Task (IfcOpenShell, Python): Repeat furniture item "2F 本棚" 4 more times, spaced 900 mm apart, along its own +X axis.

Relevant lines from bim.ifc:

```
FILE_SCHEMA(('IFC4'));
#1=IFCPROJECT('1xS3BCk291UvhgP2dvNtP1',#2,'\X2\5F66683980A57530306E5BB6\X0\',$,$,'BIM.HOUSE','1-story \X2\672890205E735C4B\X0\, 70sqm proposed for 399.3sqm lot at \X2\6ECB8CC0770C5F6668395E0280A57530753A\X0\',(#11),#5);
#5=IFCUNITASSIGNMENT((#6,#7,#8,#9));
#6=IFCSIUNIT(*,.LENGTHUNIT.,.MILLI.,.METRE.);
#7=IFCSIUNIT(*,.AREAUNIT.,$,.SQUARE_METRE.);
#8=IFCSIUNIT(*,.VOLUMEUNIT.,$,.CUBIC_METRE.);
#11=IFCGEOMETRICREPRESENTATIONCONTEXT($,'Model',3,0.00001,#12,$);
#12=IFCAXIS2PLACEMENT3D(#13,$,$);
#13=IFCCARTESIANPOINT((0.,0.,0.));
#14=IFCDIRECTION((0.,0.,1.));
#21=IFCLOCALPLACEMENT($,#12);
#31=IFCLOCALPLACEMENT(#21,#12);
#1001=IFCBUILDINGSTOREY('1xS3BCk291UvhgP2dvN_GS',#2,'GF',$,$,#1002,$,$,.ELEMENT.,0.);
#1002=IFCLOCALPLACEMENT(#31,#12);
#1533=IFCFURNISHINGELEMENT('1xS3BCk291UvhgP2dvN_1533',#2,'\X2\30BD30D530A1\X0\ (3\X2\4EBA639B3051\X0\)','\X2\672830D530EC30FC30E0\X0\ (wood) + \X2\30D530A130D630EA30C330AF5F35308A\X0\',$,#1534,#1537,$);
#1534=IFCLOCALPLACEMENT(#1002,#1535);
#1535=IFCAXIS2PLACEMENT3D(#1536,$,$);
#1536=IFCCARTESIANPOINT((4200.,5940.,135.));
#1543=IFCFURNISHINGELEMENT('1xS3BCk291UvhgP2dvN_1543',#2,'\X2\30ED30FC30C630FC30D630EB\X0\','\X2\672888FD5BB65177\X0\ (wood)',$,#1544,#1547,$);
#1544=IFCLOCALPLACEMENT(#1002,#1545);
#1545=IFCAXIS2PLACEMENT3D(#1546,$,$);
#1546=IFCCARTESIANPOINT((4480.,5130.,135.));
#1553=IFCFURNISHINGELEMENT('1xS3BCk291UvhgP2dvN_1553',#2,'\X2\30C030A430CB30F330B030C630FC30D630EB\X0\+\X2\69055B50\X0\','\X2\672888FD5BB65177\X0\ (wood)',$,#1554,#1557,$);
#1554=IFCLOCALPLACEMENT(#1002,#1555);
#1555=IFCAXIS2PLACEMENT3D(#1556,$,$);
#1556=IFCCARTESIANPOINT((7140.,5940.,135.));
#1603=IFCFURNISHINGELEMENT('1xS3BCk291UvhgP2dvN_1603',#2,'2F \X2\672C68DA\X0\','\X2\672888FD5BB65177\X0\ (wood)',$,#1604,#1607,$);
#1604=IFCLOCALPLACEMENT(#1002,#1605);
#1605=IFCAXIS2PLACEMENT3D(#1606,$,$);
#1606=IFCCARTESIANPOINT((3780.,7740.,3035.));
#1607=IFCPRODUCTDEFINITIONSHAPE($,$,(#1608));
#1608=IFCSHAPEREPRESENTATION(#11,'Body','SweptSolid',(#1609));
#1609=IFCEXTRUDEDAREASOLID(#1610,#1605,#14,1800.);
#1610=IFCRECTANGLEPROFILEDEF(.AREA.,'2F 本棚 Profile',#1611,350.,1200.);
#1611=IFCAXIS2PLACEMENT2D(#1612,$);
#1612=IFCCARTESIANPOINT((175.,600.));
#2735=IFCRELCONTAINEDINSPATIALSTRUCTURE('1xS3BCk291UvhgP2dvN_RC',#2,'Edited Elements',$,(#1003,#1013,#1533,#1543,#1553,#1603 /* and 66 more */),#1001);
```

```python
import ifcopenshell
import ifcopenshell.api.geometry
import ifcopenshell.api.root
import ifcopenshell.util.element
import ifcopenshell.util.placement

model = ifcopenshell.open("bim.ifc")


def reuse_history(source, copy):
    """copy_class also copies each property set's owner history, people and application; keep the originals."""
    for rel in copy.IsDefinedBy:
        if rel.is_a("IfcRelDefinesByProperties") and (history := rel.RelatingPropertyDefinition.OwnerHistory):
            rel.RelatingPropertyDefinition.OwnerHistory = source.OwnerHistory
            ifcopenshell.util.element.remove_deep2(model, history)


source = model.by_id(1603)
base = ifcopenshell.util.placement.get_local_placement(source.ObjectPlacement)
step = base[:3, 0] * 900.0

for i in range(1, 5):
    copy = ifcopenshell.api.root.copy_class(model, product=source)
    copy.Representation = ifcopenshell.util.element.copy_deep(
        model, source.Representation, exclude=["IfcGeometricRepresentationContext", "IfcRepresentationMap"]
    )
    reuse_history(source, copy)
    matrix = base.copy()
    matrix[:3, 3] += i * step
    print("added at", matrix[:3, 3].round(3) + 0.0)
    ifcopenshell.api.geometry.edit_object_placement(model, product=copy, matrix=matrix, is_si=False)

model.write("bim_v2.ifc")
```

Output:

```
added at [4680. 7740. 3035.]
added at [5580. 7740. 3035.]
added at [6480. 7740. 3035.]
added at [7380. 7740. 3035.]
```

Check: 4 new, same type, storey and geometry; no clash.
